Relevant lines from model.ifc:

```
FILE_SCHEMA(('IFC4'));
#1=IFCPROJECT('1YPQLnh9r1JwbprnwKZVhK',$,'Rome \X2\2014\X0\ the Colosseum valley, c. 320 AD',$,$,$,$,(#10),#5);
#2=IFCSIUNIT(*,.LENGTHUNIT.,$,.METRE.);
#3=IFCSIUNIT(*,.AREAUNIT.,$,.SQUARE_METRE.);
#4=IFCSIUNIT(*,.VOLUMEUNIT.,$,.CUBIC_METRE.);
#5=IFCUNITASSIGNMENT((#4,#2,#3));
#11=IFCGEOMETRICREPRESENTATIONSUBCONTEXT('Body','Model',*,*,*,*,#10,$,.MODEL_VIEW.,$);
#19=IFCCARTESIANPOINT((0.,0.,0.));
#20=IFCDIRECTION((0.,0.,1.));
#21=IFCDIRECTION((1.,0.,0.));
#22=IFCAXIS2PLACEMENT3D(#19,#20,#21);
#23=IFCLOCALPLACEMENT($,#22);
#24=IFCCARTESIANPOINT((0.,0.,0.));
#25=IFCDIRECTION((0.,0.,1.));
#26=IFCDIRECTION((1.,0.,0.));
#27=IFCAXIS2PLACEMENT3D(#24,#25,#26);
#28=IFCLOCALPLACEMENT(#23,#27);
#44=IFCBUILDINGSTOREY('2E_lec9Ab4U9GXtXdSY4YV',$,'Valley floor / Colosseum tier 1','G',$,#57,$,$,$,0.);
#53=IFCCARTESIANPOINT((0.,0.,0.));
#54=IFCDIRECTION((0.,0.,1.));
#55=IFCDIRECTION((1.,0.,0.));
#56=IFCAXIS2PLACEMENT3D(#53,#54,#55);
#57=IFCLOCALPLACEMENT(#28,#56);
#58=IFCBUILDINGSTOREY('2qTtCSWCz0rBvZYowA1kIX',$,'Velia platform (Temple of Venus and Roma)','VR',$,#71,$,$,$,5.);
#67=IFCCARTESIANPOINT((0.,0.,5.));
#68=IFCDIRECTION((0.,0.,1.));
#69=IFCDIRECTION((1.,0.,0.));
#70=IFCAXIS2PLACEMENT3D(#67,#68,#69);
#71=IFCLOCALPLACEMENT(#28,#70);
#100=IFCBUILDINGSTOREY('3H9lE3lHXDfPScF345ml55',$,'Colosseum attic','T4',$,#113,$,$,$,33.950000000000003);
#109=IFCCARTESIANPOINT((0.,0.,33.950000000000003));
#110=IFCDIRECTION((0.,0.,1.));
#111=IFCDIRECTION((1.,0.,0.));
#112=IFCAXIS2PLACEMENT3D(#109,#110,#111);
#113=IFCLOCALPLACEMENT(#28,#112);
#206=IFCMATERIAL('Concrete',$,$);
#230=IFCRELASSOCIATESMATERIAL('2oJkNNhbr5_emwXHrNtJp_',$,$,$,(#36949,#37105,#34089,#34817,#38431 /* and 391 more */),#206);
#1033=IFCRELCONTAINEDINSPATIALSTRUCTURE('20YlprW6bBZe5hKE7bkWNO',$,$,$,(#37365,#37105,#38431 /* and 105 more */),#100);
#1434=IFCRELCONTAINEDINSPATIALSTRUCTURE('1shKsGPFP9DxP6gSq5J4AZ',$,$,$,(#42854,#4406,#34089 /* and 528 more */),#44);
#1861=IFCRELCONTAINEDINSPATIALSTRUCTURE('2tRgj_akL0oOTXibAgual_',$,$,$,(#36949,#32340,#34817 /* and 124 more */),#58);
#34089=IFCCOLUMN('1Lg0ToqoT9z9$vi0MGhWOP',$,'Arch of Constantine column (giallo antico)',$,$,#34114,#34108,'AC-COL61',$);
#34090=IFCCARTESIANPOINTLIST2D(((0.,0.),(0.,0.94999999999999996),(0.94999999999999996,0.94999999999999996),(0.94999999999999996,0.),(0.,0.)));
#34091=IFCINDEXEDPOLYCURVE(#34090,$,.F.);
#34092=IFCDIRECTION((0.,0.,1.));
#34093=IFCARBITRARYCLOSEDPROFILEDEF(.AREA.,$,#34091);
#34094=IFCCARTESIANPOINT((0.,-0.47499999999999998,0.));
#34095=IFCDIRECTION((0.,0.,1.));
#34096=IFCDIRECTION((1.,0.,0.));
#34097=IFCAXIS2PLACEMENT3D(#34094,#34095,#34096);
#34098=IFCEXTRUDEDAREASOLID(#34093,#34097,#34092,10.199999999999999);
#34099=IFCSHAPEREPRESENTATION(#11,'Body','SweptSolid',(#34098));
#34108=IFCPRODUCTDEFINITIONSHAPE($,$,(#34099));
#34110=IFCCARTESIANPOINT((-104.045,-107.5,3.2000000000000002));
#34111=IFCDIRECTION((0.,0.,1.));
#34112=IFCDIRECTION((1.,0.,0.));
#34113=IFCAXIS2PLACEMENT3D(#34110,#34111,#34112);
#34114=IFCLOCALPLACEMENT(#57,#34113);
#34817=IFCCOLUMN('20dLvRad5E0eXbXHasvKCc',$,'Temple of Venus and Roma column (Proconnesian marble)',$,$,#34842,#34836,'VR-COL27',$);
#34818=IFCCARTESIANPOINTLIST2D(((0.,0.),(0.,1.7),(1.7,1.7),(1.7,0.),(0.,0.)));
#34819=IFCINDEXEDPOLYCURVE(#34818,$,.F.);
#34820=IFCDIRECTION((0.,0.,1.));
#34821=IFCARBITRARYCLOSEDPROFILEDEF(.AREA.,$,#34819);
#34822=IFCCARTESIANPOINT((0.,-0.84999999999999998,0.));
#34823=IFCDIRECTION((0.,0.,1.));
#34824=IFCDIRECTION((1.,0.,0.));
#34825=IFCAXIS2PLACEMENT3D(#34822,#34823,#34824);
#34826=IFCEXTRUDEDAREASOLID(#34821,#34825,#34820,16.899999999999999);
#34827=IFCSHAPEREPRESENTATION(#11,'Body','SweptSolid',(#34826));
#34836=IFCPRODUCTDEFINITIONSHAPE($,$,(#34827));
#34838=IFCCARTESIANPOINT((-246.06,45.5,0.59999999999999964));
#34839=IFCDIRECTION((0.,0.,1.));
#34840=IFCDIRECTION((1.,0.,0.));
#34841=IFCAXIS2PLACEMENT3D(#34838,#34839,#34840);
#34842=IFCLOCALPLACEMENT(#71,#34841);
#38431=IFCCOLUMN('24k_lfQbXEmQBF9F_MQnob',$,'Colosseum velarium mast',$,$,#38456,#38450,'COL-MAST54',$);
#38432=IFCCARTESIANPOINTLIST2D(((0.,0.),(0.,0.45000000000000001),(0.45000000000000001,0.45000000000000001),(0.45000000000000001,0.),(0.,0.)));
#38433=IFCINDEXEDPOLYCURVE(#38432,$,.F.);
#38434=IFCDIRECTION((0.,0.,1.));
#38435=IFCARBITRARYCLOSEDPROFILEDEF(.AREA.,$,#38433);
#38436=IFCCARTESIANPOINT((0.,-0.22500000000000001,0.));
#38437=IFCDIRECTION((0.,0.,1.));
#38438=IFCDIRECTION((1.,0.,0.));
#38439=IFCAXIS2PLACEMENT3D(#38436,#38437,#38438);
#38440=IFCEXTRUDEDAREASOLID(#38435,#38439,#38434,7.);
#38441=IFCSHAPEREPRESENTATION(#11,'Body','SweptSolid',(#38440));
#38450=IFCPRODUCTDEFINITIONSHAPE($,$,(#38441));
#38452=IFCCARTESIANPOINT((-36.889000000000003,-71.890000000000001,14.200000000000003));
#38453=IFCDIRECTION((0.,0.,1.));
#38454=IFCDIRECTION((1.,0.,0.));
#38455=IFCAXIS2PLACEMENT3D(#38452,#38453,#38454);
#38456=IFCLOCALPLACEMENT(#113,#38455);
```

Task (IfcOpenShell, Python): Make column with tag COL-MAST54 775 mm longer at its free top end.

```python
import ifcopenshell
import ifcopenshell.util.representation
import ifcopenshell.util.unit

model = ifcopenshell.open("model.ifc")
unit_scale = ifcopenshell.util.unit.calculate_unit_scale(model)

member = model.by_guid("24k_lfQbXEmQBF9F_MQnob")
change = 0.775 / unit_scale

# The extrusion runs towards the end named, so only its depth changes.
body = ifcopenshell.util.representation.get_representation(member, "Model", "Body")
solid = body.Items[0]
old_length = solid.Depth
solid.Depth += change

print(f"length {old_length:g} -> {solid.Depth:g}")

model.write("model_edited.ifc")
```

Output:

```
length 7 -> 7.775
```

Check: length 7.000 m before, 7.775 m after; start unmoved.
